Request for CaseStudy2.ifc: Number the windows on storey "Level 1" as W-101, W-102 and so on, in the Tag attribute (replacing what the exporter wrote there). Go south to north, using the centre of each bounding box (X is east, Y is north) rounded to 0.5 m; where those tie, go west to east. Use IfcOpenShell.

First a look at what the model holds.

```python
import ifcopenshell
import ifcopenshell.util.element
import ifcopenshell.util.placement

model = ifcopenshell.open("CaseStudy2.ifc")
print(model.schema)
storey = next(s for s in model.by_type("IfcBuildingStorey") if s.Name == "Level 1")
windows = [e for e in ifcopenshell.util.element.get_decomposition(storey) if e.is_a("IfcWindow")]
for e in sorted(windows, key=lambda e: e.id()):
    origin = ifcopenshell.util.placement.get_local_placement(e.ObjectPlacement)[:3, 3]
    print(e.id(), e.Tag, e.Name, origin.round(2) + 0.0, sep=" | ")
```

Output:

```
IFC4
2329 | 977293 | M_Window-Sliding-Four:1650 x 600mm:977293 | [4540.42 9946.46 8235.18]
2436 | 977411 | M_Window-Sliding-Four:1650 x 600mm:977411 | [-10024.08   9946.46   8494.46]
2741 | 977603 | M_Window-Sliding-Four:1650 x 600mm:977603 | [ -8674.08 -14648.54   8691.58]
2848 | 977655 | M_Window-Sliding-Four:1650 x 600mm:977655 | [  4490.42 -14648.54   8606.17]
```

```python
import ifcopenshell
import ifcopenshell.geom
import ifcopenshell.util.element
import ifcopenshell.util.shape

model = ifcopenshell.open("CaseStudy2.ifc")
settings = ifcopenshell.geom.settings()
settings.set("use-world-coords", True)


def centre(element):
    shape = ifcopenshell.geom.create_shape(settings, element)
    return ifcopenshell.util.shape.get_bbox_centroid(shape.geometry)


storey = next(s for s in model.by_type("IfcBuildingStorey") if s.Name == "Level 1")
windows = [e for e in ifcopenshell.util.element.get_decomposition(storey) if e.is_a("IfcWindow")]

# Insertion points can sit at a corner or the storey origin, so sort by the geometry (in metres).
centres = {e: centre(e) for e in windows}
windows.sort(key=lambda e: (round(centres[e][1] / 0.5), centres[e][0]))

for i, e in enumerate(windows, start=1):
    number = f"W-1{i:02d}"
    e.Tag = number
    print(e.id(), number)

model.write("CaseStudy2_updated.ifc")
```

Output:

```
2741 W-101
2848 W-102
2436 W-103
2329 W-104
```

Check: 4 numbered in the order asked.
